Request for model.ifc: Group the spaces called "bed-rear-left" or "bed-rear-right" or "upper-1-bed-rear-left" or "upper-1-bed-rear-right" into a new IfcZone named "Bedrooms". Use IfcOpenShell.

First a look at what the model holds.

```python
import ifcopenshell

model = ifcopenshell.open("model.ifc")
print(model.schema)
seen = {}
for space in model.by_type("IfcSpace"):
    seen[space.LongName] = seen.get(space.LongName, 0) + 1
for name, count in sorted(seen.items(), key=str):
    print(count, "x", name)
print("zones:", [z.Name for z in model.by_type("IfcZone")][:20])
```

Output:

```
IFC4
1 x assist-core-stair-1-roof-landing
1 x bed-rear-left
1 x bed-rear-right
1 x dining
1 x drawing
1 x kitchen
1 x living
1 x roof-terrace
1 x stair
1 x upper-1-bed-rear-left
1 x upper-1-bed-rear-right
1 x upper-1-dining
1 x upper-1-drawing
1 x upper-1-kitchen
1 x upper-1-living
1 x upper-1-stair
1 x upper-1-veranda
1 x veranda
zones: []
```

```python
import ifcopenshell
import ifcopenshell.api.group
import ifcopenshell.api.root

model = ifcopenshell.open("model.ifc")

names = {"bed-rear-left", "bed-rear-right", "upper-1-bed-rear-left", "upper-1-bed-rear-right"}
spaces = [s for s in model.by_type("IfcSpace") if s.LongName in names]

zone = ifcopenshell.api.root.create_entity(model, ifc_class="IfcZone", name="Bedrooms")
ifcopenshell.api.group.assign_group(model, products=spaces, group=zone)
print(len(spaces), "spaces in", zone.Name)

model.write("model_updated.ifc")
```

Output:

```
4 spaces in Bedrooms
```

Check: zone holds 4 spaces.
